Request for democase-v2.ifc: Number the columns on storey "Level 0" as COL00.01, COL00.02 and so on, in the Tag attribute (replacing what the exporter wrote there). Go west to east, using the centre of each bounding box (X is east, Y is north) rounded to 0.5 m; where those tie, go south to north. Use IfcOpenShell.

First a look at what the model holds.

```python
import ifcopenshell
import ifcopenshell.util.element
import ifcopenshell.util.placement

model = ifcopenshell.open("democase-v2.ifc")
print(model.schema)
storey = next(s for s in model.by_type("IfcBuildingStorey") if s.Name == "Level 0")
columns = [e for e in ifcopenshell.util.element.get_decomposition(storey) if e.is_a("IfcColumn")]
for e in sorted(columns, key=lambda e: e.id()):
    origin = ifcopenshell.util.placement.get_local_placement(e.ObjectPlacement)[:3, 3]
    print(e.id(), e.Tag, e.Name, origin.round(2) + 0.0, sep=" | ")
```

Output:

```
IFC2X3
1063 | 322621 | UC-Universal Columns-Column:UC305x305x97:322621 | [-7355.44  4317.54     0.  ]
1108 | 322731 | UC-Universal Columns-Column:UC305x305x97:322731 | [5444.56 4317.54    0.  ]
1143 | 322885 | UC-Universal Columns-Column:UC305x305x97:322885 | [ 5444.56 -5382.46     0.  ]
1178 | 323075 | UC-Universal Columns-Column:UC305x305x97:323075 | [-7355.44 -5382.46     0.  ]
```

```python
import ifcopenshell
import ifcopenshell.geom
import ifcopenshell.util.element
import ifcopenshell.util.shape

model = ifcopenshell.open("democase-v2.ifc")
settings = ifcopenshell.geom.settings()
settings.set("use-world-coords", True)


def centre(element):
    shape = ifcopenshell.geom.create_shape(settings, element)
    return ifcopenshell.util.shape.get_bbox_centroid(shape.geometry)


storey = next(s for s in model.by_type("IfcBuildingStorey") if s.Name == "Level 0")
columns = [e for e in ifcopenshell.util.element.get_decomposition(storey) if e.is_a("IfcColumn")]

# Insertion points can sit at a corner or the storey origin, so sort by the geometry (in metres).
centres = {e: centre(e) for e in columns}
columns.sort(key=lambda e: (round(centres[e][0] / 0.5), centres[e][1]))

for i, e in enumerate(columns, start=1):
    number = f"COL00.{i:02d}"
    e.Tag = number
    print(e.id(), number)

model.write("democase-v2_rev.ifc")
```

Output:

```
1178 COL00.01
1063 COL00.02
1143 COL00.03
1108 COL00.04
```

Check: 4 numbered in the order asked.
